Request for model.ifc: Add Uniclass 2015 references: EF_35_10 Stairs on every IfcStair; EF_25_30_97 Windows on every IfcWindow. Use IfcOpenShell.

First a look at what the model holds.

```python
import ifcopenshell

model = ifcopenshell.open("model.ifc")
print(model.schema)
print("classifications:", [c.Name for c in model.by_type("IfcClassification")])
for ifc_class in ("IfcDoor", "IfcRoof", "IfcStair", "IfcWall", "IfcWindow"):
    print(ifc_class, len(model.by_type(ifc_class)))
```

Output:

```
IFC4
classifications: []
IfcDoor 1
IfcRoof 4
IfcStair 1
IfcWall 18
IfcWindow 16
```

```python
import ifcopenshell
import ifcopenshell.api.classification

model = ifcopenshell.open("model.ifc")

system = ifcopenshell.api.classification.add_classification(model, classification="Uniclass 2015")

codes = {
    "IfcStair": ("EF_35_10", "Stairs"),
    "IfcWindow": ("EF_25_30_97", "Windows"),
}
for ifc_class, (code, name) in codes.items():
    products = model.by_type(ifc_class)
    ifcopenshell.api.classification.add_reference(
        model, products=products, classification=system, identification=code, name=name
    )
    print(code, len(products))

model.write("model_edited.ifc")
```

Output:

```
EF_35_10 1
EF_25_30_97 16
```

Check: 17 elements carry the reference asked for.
